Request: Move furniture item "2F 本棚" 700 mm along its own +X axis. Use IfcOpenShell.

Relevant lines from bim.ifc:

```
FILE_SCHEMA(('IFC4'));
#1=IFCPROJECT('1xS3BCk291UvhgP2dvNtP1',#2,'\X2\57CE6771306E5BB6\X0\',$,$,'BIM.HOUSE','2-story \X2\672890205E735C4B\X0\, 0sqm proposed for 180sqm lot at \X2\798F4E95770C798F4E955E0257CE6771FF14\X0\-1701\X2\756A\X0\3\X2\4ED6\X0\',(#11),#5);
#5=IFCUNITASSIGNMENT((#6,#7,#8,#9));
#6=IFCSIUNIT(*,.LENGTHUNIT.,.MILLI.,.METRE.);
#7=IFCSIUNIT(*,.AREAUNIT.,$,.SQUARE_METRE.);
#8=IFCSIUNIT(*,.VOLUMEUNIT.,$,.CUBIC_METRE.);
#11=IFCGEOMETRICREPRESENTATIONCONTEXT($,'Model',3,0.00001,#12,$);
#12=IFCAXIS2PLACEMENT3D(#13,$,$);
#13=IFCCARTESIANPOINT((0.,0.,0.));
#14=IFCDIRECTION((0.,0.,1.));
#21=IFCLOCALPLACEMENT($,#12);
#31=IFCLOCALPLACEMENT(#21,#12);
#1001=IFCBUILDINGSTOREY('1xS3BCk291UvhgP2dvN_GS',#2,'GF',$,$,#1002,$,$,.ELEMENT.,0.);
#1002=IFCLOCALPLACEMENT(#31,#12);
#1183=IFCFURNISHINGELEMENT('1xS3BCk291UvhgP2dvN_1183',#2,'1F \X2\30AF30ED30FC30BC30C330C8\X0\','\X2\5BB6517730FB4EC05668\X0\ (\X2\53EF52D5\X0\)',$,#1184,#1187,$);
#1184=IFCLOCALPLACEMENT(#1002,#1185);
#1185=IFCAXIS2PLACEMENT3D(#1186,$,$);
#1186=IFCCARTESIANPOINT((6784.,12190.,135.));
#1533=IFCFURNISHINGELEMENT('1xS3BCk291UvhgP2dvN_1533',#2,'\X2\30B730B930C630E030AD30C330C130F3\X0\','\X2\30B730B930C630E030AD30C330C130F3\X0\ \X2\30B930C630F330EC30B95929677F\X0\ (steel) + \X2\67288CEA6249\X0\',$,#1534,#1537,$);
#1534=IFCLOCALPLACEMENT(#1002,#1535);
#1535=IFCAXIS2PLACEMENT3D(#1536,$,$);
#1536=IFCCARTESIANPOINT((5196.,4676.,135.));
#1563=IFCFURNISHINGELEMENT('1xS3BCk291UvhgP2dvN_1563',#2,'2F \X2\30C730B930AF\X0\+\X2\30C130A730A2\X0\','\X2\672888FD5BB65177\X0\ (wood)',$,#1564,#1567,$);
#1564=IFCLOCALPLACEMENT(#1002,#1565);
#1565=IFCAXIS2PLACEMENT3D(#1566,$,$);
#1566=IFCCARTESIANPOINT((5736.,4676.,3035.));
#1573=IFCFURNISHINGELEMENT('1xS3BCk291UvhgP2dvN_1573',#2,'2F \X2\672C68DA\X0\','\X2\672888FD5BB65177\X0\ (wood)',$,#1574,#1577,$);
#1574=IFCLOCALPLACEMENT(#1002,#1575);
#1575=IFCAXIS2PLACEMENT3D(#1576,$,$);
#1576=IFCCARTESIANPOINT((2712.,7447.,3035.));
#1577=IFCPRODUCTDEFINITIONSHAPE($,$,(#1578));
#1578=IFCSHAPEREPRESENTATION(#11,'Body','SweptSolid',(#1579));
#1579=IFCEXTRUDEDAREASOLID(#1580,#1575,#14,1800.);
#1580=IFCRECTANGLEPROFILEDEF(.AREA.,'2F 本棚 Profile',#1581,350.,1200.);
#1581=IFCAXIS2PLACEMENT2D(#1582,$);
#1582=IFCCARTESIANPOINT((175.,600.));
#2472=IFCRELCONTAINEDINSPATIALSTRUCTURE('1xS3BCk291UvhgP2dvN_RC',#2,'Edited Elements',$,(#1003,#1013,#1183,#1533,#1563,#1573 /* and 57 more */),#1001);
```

```python
import ifcopenshell
import ifcopenshell.api.geometry
import ifcopenshell.util.placement
import ifcopenshell.util.unit

model = ifcopenshell.open("bim.ifc")
unit_scale = ifcopenshell.util.unit.calculate_unit_scale(model)

item = model.by_id(1573)
matrix = ifcopenshell.util.placement.get_local_placement(item.ObjectPlacement)
matrix[:3, 3] += matrix[:3, 0] * 0.7 / unit_scale
ifcopenshell.api.geometry.edit_object_placement(model, product=item, matrix=matrix, is_si=False)

print(ifcopenshell.util.placement.get_local_placement(item.ObjectPlacement).round(3) + 0.0)

model.write("bim_edited.ifc")
```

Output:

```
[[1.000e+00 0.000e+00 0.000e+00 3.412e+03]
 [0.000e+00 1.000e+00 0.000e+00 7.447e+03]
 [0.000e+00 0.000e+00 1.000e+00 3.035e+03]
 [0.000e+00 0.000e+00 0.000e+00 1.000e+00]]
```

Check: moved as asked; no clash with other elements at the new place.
